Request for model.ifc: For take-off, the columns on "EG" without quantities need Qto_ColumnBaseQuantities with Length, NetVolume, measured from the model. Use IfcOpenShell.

First a look at what the model holds.

```python
import ifcopenshell
import ifcopenshell.util.element
import ifcopenshell.util.unit

model = ifcopenshell.open("model.ifc")
print(model.schema)
for unit_type in ("LENGTHUNIT", "AREAUNIT", "VOLUMEUNIT"):
    print(unit_type, ifcopenshell.util.unit.calculate_unit_scale(model, unit_type))
storey = next(s for s in model.by_type("IfcBuildingStorey") if s.Name == "EG")
columns = [e for e in ifcopenshell.util.element.get_decomposition(storey) if e.is_a("IfcColumn")]
for e in sorted(columns, key=lambda e: e.id()):
    print(e.id(), e.is_a(), e.Name, list(ifcopenshell.util.element.get_psets(e, qtos_only=True)), sep=" | ")
```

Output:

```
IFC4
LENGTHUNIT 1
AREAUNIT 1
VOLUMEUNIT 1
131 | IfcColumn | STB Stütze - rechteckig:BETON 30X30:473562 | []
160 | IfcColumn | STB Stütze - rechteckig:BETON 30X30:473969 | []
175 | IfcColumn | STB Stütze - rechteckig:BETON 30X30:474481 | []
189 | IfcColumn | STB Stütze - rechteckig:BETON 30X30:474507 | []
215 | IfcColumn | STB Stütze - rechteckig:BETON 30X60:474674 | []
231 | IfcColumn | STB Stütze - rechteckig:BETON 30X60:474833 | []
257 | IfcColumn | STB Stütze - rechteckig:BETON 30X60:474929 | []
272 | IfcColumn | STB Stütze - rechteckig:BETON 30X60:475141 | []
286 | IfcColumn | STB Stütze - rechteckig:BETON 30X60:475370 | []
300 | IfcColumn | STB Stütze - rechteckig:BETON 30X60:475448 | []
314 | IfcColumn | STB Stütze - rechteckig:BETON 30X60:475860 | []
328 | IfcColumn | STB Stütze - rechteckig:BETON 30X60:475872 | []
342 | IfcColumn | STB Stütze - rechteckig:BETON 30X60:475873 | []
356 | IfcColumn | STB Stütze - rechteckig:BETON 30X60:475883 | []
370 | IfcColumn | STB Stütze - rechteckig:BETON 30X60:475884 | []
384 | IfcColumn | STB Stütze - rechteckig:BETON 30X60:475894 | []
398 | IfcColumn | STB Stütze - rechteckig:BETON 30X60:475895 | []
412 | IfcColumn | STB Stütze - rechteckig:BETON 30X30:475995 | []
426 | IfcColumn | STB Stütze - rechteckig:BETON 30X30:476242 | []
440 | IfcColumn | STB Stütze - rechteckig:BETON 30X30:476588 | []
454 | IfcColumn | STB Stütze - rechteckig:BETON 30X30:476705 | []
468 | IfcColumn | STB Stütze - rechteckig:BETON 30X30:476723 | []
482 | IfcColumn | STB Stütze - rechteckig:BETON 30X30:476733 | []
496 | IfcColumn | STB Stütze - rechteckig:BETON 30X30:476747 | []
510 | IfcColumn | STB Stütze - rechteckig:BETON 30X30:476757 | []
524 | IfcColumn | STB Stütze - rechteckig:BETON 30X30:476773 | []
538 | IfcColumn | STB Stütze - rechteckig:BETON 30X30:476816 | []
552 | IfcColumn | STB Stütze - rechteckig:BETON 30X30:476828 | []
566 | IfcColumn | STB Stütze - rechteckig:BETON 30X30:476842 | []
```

```python
import ifcopenshell
import ifcopenshell.api.pset
import ifcopenshell.geom
import ifcopenshell.util.element
import ifcopenshell.util.shape
import ifcopenshell.util.unit

model = ifcopenshell.open("model.ifc")
unit_scale = ifcopenshell.util.unit.calculate_unit_scale(model)
volume_scale = ifcopenshell.util.unit.calculate_unit_scale(model, "VOLUMEUNIT")
settings = ifcopenshell.geom.settings()

storey = next(s for s in model.by_type("IfcBuildingStorey") if s.Name == "EG")
columns = [e for e in ifcopenshell.util.element.get_decomposition(storey) if e.is_a("IfcColumn")]

for e in sorted(columns, key=lambda e: e.id()):
    if ifcopenshell.util.element.get_psets(e, qtos_only=True, should_inherit=False):
        continue
    # Geometry comes back in metres, in the element's own axes.
    shape = ifcopenshell.geom.create_shape(settings, e)
    values = {
        "Length": ifcopenshell.util.shape.get_z(shape.geometry) / unit_scale,
        "NetVolume": ifcopenshell.util.shape.get_volume(shape.geometry) / volume_scale,
    }
    qto = ifcopenshell.api.pset.add_qto(model, product=e, name="Qto_ColumnBaseQuantities")
    ifcopenshell.api.pset.edit_qto(model, qto=qto, properties=values)
    print(e.id(), {k: round(v, 3) for k, v in values.items()})

model.write("model_edited.ifc")
```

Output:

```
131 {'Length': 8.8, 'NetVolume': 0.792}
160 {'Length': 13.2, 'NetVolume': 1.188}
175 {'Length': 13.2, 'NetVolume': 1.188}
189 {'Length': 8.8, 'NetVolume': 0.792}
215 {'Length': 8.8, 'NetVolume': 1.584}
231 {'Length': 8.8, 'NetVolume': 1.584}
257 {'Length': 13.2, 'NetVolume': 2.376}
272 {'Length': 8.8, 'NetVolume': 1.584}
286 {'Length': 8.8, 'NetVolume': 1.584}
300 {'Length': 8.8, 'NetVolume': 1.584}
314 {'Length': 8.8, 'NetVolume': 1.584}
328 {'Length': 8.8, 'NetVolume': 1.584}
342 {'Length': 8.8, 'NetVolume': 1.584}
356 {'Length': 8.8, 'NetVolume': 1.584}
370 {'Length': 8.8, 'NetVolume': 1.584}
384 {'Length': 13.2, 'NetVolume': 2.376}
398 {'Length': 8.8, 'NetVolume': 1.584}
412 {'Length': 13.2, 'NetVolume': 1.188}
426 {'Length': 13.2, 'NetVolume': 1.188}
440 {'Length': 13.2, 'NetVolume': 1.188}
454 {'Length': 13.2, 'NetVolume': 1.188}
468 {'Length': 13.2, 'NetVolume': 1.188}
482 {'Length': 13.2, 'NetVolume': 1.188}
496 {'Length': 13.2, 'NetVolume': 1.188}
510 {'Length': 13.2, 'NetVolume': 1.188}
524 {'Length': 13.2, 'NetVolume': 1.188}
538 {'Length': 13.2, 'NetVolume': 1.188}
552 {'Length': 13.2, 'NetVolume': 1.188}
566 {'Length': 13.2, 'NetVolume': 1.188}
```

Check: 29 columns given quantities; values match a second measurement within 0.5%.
